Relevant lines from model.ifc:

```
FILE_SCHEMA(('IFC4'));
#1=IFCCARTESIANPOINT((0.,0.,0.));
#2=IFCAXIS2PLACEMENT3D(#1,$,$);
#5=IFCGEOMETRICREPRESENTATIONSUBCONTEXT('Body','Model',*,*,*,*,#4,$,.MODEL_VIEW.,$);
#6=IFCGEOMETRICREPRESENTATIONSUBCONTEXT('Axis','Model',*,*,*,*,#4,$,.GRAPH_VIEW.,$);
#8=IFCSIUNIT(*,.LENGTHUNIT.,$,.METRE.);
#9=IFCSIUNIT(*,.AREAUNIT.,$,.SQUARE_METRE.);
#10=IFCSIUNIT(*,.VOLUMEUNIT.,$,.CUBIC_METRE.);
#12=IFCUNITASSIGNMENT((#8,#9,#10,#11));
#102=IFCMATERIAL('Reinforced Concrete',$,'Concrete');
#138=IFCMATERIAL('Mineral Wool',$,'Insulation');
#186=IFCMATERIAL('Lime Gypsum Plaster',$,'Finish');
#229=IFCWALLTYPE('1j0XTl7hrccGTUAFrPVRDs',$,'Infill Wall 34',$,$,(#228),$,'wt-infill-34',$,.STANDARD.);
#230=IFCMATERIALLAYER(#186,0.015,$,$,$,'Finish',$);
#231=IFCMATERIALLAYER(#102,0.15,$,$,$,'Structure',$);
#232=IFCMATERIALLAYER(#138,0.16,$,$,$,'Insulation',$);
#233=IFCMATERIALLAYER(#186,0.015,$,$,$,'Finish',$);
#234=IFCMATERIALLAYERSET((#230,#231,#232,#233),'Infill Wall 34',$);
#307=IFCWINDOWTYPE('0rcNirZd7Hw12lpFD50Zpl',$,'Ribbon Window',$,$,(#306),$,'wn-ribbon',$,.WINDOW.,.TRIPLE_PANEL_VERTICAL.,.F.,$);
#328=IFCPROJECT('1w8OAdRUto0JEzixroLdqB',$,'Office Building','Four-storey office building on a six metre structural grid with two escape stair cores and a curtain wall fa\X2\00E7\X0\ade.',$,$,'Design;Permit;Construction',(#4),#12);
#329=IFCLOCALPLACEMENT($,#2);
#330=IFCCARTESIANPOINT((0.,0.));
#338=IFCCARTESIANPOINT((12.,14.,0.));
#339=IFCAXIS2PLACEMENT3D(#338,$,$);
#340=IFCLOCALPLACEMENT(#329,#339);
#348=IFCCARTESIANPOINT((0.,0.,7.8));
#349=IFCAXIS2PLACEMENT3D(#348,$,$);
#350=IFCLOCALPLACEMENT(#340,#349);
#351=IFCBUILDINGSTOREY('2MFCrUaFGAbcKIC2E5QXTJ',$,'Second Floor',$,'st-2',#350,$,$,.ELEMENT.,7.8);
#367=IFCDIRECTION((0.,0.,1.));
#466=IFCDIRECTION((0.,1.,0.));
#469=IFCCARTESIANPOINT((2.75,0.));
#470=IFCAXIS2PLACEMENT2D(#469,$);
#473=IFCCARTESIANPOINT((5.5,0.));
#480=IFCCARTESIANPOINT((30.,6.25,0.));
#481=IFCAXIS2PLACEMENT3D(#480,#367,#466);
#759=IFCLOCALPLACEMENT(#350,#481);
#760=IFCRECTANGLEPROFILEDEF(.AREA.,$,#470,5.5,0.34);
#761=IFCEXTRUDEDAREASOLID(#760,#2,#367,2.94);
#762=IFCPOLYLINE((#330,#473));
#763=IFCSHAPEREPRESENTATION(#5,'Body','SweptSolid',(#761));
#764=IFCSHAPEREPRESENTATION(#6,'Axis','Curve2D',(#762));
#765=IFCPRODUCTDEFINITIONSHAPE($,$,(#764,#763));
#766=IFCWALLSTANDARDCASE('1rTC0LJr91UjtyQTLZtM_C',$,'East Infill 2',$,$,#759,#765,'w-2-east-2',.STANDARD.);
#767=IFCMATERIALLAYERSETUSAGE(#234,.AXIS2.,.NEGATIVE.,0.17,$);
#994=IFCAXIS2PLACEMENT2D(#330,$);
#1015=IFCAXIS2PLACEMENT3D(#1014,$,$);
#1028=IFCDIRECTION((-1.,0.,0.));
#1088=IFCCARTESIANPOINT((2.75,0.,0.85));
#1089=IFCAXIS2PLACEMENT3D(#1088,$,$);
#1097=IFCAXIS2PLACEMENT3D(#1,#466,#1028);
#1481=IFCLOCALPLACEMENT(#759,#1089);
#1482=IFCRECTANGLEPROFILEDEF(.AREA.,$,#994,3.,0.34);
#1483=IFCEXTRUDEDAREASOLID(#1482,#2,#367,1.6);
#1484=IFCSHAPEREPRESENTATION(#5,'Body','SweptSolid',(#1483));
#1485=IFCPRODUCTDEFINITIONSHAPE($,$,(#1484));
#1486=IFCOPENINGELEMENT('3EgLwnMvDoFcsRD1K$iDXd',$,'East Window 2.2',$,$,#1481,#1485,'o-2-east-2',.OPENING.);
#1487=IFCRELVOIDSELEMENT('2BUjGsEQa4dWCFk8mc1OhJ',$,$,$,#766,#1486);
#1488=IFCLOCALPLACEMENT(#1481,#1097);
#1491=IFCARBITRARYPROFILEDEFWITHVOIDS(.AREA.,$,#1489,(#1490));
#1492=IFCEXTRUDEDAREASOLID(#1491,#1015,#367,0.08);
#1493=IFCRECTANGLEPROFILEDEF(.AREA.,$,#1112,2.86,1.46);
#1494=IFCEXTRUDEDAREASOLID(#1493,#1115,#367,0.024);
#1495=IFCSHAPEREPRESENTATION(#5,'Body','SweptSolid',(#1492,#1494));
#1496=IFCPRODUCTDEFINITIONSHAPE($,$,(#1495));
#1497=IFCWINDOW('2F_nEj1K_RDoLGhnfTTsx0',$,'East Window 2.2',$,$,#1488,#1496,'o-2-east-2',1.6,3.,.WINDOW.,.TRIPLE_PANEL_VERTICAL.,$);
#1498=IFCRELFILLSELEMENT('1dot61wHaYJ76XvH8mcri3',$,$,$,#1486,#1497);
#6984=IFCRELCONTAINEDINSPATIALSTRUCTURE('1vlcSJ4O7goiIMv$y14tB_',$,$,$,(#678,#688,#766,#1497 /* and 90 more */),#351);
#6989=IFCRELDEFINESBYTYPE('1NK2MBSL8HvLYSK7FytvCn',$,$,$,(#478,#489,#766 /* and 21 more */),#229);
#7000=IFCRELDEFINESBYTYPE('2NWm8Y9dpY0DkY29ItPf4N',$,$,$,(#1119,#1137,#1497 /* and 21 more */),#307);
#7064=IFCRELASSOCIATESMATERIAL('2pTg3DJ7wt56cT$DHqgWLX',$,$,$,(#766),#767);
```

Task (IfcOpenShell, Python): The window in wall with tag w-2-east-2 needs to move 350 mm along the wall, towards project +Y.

```python
import ifcopenshell
import ifcopenshell.api.geometry
import ifcopenshell.util.placement
import ifcopenshell.util.unit

model = ifcopenshell.open("model.ifc")
unit_scale = ifcopenshell.util.unit.calculate_unit_scale(model)

window = model.by_guid("2F_nEj1K_RDoLGhnfTTsx0")
opening = window.FillsVoids[0].RelatingOpeningElement
wall = opening.VoidsElements[0].RelatingBuildingElement

wall_matrix = ifcopenshell.util.placement.get_local_placement(wall.ObjectPlacement)
shift = wall_matrix[:3, 0] * 0.35 / unit_scale
before = ifcopenshell.util.placement.get_local_placement(window.ObjectPlacement)[:3, 3].copy()

# The window is placed relative to its opening, so it follows when the opening moves.
matrix = ifcopenshell.util.placement.get_local_placement(opening.ObjectPlacement)
matrix[:3, 3] += shift
ifcopenshell.api.geometry.edit_object_placement(
    model, product=opening, matrix=matrix, is_si=False, should_transform_children=True
)

after = ifcopenshell.util.placement.get_local_placement(window.ObjectPlacement)[:3, 3]
print("window moved by", (after - before).round(3) + 0.0)

model.write("model_edited.ifc")
```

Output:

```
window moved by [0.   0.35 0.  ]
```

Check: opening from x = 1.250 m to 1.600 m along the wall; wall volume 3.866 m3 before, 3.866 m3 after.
